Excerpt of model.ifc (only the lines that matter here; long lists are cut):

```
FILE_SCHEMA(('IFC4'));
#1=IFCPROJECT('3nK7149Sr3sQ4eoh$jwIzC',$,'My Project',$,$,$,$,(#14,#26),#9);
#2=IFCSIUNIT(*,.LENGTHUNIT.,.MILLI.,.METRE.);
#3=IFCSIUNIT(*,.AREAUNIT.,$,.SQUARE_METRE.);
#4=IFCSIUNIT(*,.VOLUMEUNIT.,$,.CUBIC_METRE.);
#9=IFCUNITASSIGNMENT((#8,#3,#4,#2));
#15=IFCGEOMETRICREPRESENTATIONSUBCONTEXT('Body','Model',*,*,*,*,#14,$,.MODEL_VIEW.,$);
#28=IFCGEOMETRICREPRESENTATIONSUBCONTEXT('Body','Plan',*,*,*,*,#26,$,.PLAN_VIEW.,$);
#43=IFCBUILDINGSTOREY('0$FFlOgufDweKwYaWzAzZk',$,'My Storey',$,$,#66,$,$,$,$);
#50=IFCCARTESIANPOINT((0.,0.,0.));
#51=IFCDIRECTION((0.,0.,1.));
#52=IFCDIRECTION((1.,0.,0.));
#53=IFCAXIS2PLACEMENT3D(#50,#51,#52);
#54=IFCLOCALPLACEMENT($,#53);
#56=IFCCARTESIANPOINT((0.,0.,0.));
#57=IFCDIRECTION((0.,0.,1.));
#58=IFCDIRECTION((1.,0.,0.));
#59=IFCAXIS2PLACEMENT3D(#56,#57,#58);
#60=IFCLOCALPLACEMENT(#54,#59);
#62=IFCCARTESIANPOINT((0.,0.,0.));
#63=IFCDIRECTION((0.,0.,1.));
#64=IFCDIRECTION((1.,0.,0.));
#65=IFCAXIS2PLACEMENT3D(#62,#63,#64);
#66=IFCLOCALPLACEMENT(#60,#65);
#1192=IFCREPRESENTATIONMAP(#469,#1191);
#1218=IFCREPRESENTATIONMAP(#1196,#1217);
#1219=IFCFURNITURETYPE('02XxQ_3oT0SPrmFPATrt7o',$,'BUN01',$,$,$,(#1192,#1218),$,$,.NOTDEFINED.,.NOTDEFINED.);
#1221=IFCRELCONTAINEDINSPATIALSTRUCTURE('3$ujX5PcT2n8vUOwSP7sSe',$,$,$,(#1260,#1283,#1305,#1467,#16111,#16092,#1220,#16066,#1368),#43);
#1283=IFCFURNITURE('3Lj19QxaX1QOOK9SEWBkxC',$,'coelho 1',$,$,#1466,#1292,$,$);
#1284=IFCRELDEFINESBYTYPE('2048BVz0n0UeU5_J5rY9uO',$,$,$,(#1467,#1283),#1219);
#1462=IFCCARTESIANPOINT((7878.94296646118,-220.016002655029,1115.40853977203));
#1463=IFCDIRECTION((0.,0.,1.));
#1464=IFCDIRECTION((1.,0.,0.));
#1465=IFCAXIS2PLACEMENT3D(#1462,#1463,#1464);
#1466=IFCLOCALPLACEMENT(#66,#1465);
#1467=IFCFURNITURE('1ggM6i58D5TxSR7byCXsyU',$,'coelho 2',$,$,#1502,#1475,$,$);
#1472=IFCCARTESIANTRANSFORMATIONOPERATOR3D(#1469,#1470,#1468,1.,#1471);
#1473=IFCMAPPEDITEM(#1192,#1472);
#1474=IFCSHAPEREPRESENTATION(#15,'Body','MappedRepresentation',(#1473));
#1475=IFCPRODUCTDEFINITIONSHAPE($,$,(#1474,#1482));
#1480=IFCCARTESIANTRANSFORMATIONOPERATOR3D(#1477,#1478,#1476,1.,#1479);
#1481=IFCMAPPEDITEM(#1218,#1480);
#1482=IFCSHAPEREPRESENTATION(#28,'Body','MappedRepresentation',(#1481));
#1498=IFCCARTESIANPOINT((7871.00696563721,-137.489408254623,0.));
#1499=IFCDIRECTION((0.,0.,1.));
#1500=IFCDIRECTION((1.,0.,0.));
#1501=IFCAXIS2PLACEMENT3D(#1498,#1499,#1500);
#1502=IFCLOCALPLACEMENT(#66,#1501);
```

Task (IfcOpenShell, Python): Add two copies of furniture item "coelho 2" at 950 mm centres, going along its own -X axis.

```python
import ifcopenshell
import ifcopenshell.api.geometry
import ifcopenshell.api.root
import ifcopenshell.util.element
import ifcopenshell.util.placement

model = ifcopenshell.open("model.ifc")

source = model.by_guid("1ggM6i58D5TxSR7byCXsyU")
base = ifcopenshell.util.placement.get_local_placement(source.ObjectPlacement)
step = -base[:3, 0] * 950.0

for i in range(1, 3):
    copy = ifcopenshell.api.root.copy_class(model, product=source)
    copy.Representation = ifcopenshell.util.element.copy_deep(
        model, source.Representation, exclude=["IfcGeometricRepresentationContext", "IfcRepresentationMap"]
    )
    matrix = base.copy()
    matrix[:3, 3] += i * step
    print("added at", matrix[:3, 3].round(3) + 0.0)
    ifcopenshell.api.geometry.edit_object_placement(model, product=copy, matrix=matrix, is_si=False)

model.write("model_rev.ifc")
```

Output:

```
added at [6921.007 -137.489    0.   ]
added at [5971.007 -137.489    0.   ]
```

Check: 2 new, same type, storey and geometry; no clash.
